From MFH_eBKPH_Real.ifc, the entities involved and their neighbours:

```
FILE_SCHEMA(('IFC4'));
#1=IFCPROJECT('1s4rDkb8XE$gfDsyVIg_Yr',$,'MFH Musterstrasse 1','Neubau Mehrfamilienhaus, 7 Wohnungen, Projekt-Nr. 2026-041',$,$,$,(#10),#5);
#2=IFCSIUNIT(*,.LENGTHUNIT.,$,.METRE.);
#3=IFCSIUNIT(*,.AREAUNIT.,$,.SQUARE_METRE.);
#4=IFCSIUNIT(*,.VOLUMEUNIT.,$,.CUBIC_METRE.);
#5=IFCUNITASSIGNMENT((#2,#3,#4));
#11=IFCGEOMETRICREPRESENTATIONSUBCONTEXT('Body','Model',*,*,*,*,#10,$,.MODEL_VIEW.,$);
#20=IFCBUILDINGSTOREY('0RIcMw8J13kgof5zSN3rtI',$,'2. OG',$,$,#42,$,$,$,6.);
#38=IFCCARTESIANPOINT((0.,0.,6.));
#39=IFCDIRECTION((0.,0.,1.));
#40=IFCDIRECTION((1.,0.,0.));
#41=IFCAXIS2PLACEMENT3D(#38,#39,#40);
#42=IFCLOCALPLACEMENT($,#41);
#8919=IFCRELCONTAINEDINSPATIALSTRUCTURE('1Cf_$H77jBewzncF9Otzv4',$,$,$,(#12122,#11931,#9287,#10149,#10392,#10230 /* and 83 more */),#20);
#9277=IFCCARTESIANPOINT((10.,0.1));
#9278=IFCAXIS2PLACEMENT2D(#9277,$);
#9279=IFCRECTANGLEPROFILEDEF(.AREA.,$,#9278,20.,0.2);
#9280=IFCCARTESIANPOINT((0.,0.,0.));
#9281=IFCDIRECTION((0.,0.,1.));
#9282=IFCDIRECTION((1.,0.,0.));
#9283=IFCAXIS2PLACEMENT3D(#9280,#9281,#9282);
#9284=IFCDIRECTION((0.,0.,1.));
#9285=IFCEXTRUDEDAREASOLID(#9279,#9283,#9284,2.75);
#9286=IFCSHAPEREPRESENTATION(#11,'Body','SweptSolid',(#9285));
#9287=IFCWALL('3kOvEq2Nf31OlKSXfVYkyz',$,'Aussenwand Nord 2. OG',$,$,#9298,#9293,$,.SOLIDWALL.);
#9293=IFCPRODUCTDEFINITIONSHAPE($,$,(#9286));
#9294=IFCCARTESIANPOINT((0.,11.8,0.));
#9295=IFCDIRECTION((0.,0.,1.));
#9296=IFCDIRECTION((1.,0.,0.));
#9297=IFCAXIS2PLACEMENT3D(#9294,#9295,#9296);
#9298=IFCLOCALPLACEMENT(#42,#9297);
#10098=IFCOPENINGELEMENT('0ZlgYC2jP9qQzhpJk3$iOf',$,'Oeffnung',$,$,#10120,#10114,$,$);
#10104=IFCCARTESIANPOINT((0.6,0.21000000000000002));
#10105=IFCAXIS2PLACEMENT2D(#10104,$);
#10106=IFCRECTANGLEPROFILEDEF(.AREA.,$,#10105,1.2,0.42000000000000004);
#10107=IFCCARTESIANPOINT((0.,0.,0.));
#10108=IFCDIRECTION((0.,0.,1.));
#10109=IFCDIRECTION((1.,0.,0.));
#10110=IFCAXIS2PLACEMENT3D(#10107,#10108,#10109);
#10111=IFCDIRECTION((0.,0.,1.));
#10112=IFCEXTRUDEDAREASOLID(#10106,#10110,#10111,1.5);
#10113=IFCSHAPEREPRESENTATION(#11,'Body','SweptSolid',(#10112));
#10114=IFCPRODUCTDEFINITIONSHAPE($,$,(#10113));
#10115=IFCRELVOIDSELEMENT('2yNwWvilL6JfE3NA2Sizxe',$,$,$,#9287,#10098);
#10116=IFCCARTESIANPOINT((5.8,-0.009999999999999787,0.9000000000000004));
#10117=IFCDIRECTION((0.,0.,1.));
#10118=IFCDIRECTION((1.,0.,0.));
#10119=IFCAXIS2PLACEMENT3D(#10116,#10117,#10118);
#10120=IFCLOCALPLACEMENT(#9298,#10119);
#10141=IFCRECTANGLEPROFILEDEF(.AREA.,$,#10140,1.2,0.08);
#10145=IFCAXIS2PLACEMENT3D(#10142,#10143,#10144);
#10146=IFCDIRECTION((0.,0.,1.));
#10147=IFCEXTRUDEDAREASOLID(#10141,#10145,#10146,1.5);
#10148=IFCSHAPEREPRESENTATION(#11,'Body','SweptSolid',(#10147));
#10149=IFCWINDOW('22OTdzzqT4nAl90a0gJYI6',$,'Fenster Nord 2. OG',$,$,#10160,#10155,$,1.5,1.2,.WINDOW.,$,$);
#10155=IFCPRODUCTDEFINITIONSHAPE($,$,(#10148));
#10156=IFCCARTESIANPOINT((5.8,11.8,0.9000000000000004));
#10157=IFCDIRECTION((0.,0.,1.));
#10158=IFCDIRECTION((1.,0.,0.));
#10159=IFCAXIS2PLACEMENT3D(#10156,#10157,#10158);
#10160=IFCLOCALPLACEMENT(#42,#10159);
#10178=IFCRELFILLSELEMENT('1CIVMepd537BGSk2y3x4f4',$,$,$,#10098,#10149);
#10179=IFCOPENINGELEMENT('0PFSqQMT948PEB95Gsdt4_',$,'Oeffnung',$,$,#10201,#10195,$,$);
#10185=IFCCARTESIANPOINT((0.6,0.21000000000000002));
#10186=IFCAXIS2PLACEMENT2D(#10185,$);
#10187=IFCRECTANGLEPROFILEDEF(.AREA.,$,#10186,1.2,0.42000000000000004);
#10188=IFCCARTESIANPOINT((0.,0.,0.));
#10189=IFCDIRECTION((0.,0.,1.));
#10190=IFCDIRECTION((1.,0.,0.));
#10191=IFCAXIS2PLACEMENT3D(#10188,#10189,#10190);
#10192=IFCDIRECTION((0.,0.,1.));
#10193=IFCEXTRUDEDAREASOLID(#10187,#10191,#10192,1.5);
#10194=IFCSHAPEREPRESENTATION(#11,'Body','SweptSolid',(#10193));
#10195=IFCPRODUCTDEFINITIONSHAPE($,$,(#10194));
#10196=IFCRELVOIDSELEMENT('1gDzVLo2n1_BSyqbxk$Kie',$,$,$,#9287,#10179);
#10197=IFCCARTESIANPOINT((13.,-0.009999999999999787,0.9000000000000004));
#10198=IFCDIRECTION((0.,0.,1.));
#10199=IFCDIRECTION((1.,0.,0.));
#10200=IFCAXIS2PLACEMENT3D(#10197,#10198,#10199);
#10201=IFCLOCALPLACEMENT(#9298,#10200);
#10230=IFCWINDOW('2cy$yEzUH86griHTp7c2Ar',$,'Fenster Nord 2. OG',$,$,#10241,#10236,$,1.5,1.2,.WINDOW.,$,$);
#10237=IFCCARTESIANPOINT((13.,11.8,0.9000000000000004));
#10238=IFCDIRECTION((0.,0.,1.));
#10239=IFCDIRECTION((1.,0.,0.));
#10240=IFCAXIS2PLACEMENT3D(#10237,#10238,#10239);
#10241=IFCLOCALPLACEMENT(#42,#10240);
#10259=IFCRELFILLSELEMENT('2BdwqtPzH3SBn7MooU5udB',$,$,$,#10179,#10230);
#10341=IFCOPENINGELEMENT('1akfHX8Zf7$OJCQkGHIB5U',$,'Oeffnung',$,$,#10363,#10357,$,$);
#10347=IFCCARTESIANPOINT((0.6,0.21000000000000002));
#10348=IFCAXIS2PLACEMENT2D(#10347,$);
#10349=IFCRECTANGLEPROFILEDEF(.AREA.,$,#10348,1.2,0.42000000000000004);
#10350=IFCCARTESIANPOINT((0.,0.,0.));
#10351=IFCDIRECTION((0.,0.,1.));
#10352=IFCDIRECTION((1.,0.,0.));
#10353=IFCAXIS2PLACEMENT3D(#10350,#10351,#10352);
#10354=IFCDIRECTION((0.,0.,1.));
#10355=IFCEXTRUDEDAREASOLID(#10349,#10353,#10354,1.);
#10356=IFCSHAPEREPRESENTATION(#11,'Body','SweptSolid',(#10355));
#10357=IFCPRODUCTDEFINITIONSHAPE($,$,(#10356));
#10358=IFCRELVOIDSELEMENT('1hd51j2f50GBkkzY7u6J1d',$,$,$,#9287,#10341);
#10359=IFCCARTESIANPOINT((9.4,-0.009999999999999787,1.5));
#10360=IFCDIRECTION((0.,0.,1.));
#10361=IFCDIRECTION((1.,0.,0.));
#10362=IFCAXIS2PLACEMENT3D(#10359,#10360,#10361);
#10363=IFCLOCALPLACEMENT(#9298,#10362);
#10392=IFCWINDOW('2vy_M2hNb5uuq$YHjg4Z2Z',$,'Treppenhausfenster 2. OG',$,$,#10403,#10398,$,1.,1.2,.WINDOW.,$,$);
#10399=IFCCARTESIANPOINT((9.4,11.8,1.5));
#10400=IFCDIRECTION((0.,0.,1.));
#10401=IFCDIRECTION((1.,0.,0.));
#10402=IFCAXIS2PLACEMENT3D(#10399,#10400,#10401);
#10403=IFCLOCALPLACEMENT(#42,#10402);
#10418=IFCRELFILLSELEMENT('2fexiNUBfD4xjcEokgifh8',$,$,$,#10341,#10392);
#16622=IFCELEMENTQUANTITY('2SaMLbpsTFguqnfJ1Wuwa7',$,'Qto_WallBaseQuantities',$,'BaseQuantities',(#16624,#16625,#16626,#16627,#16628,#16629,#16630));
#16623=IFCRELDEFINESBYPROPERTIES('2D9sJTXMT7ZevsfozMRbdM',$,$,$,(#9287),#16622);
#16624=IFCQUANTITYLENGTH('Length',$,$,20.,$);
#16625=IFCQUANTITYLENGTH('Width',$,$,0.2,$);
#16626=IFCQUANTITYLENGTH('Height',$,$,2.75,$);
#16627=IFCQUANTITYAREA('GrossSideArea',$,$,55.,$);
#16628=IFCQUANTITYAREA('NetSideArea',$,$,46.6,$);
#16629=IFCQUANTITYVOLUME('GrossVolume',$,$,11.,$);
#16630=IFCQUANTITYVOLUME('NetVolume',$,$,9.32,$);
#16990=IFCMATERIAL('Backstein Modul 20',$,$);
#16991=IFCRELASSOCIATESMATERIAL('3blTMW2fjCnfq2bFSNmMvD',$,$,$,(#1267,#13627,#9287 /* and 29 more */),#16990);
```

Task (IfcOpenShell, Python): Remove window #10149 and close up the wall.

```python
import ifcopenshell
import ifcopenshell.api.feature
import ifcopenshell.api.pset
import ifcopenshell.api.root
import ifcopenshell.geom
import ifcopenshell.util.element
import ifcopenshell.util.shape
import ifcopenshell.util.unit

model = ifcopenshell.open("MFH_eBKPH_Real.ifc")
area_scale = ifcopenshell.util.unit.calculate_unit_scale(model, "AREAUNIT")
volume_scale = ifcopenshell.util.unit.calculate_unit_scale(model, "VOLUMEUNIT")
settings = ifcopenshell.geom.settings()


def volume(element):
    """Net volume in cubic metres, openings subtracted."""
    shape = ifcopenshell.geom.create_shape(settings, element)
    return ifcopenshell.util.shape.get_volume(shape.geometry)


window = model.by_id(10149)
opening = window.FillsVoids[0].RelatingOpeningElement
wall = opening.VoidsElements[0].RelatingBuildingElement
before = volume(wall)

ifcopenshell.api.root.remove_product(model, product=window)
ifcopenshell.api.feature.remove_feature(model, feature=opening)

after = volume(wall)
thickness = 0.2  # wall thickness in metres

# Update the wall's stored quantities.
qto = model.by_id(ifcopenshell.util.element.get_pset(wall, "Qto_WallBaseQuantities", should_inherit=False)["id"])
ifcopenshell.api.pset.edit_qto(model, qto=qto, properties={
    "NetSideArea": after / thickness / area_scale,
    "NetVolume": after / volume_scale,
})

print(f"wall volume {before:.3f} -> {after:.3f} m3")

model.write("MFH_eBKPH_Real_rev.ifc")
```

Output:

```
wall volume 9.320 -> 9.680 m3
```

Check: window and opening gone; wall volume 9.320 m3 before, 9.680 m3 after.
